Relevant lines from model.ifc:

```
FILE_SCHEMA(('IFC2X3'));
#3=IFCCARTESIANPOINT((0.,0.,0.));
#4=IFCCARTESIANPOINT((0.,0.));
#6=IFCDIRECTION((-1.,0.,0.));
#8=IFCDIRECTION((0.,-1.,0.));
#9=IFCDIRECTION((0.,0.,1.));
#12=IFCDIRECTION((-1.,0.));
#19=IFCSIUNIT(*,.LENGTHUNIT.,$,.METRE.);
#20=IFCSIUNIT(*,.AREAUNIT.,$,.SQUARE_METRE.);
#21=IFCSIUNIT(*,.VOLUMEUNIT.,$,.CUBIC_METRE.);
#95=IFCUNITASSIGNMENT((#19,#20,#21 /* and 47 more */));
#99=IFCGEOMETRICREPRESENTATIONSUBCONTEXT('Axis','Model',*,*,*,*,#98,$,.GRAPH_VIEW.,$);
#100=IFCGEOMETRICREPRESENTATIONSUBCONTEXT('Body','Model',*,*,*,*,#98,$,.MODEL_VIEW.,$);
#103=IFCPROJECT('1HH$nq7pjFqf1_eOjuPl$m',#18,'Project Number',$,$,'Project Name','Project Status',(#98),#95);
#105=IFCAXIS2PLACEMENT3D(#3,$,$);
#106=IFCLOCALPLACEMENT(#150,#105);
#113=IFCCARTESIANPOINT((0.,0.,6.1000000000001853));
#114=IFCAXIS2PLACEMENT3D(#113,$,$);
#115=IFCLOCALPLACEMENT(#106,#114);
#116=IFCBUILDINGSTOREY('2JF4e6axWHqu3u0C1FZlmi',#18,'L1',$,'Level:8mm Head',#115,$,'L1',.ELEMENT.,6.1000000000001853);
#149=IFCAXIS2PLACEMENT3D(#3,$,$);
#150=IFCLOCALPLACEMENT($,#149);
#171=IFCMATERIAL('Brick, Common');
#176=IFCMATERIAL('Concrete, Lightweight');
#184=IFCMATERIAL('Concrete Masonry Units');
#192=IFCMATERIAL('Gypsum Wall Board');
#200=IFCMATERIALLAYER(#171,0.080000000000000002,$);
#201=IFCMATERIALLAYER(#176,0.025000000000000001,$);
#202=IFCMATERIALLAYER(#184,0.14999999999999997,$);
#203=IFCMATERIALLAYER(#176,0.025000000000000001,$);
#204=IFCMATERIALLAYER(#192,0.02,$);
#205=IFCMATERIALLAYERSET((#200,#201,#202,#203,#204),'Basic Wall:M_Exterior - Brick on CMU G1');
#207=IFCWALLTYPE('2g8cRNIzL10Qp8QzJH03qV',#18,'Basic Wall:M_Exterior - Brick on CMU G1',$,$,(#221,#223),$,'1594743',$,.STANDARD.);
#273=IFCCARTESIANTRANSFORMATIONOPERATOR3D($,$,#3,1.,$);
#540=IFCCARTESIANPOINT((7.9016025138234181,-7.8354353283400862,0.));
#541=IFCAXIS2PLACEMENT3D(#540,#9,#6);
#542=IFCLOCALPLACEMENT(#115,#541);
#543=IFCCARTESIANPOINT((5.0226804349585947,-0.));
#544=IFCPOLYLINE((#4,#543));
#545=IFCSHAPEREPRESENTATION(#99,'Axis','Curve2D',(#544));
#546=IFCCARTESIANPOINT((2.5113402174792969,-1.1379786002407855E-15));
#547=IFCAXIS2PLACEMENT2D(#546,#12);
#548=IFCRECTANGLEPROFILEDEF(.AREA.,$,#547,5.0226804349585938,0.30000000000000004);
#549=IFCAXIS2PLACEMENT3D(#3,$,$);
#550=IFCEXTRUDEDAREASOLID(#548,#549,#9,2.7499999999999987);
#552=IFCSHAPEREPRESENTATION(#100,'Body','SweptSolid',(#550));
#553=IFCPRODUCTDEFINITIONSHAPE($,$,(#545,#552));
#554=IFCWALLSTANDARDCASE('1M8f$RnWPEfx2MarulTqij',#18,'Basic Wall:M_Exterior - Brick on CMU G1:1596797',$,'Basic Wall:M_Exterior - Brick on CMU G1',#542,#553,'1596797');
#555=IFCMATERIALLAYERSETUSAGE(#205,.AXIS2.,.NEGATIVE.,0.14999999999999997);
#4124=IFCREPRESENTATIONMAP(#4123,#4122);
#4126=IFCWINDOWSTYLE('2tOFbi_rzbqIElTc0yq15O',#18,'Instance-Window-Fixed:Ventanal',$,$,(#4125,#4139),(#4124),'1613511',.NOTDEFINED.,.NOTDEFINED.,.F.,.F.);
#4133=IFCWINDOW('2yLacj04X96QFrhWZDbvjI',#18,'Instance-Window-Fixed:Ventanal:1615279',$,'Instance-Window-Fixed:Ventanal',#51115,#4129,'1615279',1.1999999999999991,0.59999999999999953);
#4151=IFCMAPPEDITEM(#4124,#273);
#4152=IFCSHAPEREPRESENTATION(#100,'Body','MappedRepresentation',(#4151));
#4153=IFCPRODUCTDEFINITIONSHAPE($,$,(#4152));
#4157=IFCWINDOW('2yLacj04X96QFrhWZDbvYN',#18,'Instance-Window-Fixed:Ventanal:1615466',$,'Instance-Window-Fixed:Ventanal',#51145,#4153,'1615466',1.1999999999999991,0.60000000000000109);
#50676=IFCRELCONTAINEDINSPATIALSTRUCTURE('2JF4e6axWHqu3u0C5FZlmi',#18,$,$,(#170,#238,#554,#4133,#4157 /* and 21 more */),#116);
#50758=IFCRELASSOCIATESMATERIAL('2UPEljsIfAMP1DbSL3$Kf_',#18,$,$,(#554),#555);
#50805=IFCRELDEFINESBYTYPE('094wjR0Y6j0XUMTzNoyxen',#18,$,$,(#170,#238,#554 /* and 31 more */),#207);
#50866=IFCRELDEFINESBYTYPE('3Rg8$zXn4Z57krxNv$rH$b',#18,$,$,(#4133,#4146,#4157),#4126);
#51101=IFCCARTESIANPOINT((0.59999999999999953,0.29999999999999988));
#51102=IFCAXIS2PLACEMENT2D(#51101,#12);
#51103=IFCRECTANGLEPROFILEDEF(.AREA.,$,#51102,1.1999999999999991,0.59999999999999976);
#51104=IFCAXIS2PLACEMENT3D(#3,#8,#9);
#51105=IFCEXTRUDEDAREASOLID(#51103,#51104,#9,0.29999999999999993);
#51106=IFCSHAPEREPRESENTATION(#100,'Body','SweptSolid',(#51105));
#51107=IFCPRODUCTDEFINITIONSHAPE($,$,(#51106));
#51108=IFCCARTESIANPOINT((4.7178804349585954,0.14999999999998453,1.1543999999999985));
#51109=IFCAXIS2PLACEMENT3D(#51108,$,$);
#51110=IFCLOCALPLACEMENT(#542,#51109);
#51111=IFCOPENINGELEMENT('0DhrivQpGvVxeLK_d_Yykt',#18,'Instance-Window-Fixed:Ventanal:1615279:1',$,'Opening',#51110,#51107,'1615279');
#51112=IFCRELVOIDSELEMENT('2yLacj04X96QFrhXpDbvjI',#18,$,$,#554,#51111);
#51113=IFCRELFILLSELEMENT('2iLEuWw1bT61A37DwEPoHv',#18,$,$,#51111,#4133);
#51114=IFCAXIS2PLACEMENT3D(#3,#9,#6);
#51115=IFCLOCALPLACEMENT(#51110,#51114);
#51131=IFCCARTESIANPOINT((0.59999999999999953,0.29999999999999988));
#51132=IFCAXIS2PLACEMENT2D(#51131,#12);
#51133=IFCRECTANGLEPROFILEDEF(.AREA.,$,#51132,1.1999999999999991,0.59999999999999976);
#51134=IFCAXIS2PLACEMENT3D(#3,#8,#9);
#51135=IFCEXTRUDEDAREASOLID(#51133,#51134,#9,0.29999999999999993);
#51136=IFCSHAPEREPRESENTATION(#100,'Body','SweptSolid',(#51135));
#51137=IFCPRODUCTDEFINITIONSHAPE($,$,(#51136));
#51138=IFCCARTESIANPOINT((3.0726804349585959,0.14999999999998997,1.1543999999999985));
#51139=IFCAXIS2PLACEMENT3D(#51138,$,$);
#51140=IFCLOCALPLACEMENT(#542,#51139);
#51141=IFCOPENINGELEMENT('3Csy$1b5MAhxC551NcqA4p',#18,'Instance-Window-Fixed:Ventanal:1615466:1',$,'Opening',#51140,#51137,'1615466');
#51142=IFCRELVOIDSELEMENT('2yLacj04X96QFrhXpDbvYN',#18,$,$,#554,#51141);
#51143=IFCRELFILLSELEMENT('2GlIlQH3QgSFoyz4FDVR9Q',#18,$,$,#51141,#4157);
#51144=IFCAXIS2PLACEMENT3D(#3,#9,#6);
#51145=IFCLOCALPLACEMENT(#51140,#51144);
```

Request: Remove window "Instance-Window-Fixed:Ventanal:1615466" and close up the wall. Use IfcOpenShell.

```python
import ifcopenshell
import ifcopenshell.api.feature
import ifcopenshell.api.root
import ifcopenshell.geom
import ifcopenshell.util.shape

model = ifcopenshell.open("model.ifc")
settings = ifcopenshell.geom.settings()


def volume(element):
    """Net volume in cubic metres, openings subtracted."""
    shape = ifcopenshell.geom.create_shape(settings, element)
    return ifcopenshell.util.shape.get_volume(shape.geometry)


window = model.by_guid("2yLacj04X96QFrhWZDbvYN")
opening = window.FillsVoids[0].RelatingOpeningElement
wall = opening.VoidsElements[0].RelatingBuildingElement
before = volume(wall)

ifcopenshell.api.root.remove_product(model, product=window)
ifcopenshell.api.feature.remove_feature(model, feature=opening)

after = volume(wall)

print(f"wall volume {before:.3f} -> {after:.3f} m3")

model.write("model_v2.ifc")
```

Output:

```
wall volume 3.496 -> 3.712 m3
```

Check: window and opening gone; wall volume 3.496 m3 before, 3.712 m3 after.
